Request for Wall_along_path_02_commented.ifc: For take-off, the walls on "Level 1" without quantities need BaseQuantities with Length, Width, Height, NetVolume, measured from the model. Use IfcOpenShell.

First a look at what the model holds.

```python
import ifcopenshell
import ifcopenshell.util.element
import ifcopenshell.util.unit

model = ifcopenshell.open("Wall_along_path_02_commented.ifc")
print(model.schema)
for unit_type in ("LENGTHUNIT", "AREAUNIT", "VOLUMEUNIT"):
    print(unit_type, ifcopenshell.util.unit.calculate_unit_scale(model, unit_type))
storey = next(s for s in model.by_type("IfcBuildingStorey") if s.Name == "Level 1")
walls = [e for e in ifcopenshell.util.element.get_decomposition(storey) if e.is_a("IfcWall")]
for e in sorted(walls, key=lambda e: e.id()):
    print(e.id(), e.is_a(), e.Name, list(ifcopenshell.util.element.get_psets(e, qtos_only=True)), sep=" | ")
```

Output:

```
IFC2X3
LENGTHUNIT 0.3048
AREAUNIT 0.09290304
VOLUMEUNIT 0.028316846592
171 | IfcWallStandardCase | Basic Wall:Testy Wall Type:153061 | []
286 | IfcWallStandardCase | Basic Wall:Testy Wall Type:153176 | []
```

```python
import ifcopenshell
import ifcopenshell.api.pset
import ifcopenshell.geom
import ifcopenshell.util.element
import ifcopenshell.util.shape
import ifcopenshell.util.unit

model = ifcopenshell.open("Wall_along_path_02_commented.ifc")
unit_scale = ifcopenshell.util.unit.calculate_unit_scale(model)
volume_scale = ifcopenshell.util.unit.calculate_unit_scale(model, "VOLUMEUNIT")
settings = ifcopenshell.geom.settings()

storey = next(s for s in model.by_type("IfcBuildingStorey") if s.Name == "Level 1")
walls = [e for e in ifcopenshell.util.element.get_decomposition(storey) if e.is_a("IfcWall")]

for e in sorted(walls, key=lambda e: e.id()):
    if ifcopenshell.util.element.get_psets(e, qtos_only=True, should_inherit=False):
        continue
    # Geometry comes back in metres, in the element's own axes.
    shape = ifcopenshell.geom.create_shape(settings, e)
    values = {
        "Length": ifcopenshell.util.shape.get_x(shape.geometry) / unit_scale,
        "Width": ifcopenshell.util.shape.get_y(shape.geometry) / unit_scale,
        "Height": ifcopenshell.util.shape.get_z(shape.geometry) / unit_scale,
        "NetVolume": ifcopenshell.util.shape.get_volume(shape.geometry) / volume_scale,
    }
    qto = ifcopenshell.api.pset.add_qto(model, product=e, name="BaseQuantities")
    ifcopenshell.api.pset.edit_qto(model, qto=qto, properties=values)
    print(e.id(), {k: round(v, 3) for k, v in values.items()})

model.write("Wall_along_path_02_commented_edited.ifc")
```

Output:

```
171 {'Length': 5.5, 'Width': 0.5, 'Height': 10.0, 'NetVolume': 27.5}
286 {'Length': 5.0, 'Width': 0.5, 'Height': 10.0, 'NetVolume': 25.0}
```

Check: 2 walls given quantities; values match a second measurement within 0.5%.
